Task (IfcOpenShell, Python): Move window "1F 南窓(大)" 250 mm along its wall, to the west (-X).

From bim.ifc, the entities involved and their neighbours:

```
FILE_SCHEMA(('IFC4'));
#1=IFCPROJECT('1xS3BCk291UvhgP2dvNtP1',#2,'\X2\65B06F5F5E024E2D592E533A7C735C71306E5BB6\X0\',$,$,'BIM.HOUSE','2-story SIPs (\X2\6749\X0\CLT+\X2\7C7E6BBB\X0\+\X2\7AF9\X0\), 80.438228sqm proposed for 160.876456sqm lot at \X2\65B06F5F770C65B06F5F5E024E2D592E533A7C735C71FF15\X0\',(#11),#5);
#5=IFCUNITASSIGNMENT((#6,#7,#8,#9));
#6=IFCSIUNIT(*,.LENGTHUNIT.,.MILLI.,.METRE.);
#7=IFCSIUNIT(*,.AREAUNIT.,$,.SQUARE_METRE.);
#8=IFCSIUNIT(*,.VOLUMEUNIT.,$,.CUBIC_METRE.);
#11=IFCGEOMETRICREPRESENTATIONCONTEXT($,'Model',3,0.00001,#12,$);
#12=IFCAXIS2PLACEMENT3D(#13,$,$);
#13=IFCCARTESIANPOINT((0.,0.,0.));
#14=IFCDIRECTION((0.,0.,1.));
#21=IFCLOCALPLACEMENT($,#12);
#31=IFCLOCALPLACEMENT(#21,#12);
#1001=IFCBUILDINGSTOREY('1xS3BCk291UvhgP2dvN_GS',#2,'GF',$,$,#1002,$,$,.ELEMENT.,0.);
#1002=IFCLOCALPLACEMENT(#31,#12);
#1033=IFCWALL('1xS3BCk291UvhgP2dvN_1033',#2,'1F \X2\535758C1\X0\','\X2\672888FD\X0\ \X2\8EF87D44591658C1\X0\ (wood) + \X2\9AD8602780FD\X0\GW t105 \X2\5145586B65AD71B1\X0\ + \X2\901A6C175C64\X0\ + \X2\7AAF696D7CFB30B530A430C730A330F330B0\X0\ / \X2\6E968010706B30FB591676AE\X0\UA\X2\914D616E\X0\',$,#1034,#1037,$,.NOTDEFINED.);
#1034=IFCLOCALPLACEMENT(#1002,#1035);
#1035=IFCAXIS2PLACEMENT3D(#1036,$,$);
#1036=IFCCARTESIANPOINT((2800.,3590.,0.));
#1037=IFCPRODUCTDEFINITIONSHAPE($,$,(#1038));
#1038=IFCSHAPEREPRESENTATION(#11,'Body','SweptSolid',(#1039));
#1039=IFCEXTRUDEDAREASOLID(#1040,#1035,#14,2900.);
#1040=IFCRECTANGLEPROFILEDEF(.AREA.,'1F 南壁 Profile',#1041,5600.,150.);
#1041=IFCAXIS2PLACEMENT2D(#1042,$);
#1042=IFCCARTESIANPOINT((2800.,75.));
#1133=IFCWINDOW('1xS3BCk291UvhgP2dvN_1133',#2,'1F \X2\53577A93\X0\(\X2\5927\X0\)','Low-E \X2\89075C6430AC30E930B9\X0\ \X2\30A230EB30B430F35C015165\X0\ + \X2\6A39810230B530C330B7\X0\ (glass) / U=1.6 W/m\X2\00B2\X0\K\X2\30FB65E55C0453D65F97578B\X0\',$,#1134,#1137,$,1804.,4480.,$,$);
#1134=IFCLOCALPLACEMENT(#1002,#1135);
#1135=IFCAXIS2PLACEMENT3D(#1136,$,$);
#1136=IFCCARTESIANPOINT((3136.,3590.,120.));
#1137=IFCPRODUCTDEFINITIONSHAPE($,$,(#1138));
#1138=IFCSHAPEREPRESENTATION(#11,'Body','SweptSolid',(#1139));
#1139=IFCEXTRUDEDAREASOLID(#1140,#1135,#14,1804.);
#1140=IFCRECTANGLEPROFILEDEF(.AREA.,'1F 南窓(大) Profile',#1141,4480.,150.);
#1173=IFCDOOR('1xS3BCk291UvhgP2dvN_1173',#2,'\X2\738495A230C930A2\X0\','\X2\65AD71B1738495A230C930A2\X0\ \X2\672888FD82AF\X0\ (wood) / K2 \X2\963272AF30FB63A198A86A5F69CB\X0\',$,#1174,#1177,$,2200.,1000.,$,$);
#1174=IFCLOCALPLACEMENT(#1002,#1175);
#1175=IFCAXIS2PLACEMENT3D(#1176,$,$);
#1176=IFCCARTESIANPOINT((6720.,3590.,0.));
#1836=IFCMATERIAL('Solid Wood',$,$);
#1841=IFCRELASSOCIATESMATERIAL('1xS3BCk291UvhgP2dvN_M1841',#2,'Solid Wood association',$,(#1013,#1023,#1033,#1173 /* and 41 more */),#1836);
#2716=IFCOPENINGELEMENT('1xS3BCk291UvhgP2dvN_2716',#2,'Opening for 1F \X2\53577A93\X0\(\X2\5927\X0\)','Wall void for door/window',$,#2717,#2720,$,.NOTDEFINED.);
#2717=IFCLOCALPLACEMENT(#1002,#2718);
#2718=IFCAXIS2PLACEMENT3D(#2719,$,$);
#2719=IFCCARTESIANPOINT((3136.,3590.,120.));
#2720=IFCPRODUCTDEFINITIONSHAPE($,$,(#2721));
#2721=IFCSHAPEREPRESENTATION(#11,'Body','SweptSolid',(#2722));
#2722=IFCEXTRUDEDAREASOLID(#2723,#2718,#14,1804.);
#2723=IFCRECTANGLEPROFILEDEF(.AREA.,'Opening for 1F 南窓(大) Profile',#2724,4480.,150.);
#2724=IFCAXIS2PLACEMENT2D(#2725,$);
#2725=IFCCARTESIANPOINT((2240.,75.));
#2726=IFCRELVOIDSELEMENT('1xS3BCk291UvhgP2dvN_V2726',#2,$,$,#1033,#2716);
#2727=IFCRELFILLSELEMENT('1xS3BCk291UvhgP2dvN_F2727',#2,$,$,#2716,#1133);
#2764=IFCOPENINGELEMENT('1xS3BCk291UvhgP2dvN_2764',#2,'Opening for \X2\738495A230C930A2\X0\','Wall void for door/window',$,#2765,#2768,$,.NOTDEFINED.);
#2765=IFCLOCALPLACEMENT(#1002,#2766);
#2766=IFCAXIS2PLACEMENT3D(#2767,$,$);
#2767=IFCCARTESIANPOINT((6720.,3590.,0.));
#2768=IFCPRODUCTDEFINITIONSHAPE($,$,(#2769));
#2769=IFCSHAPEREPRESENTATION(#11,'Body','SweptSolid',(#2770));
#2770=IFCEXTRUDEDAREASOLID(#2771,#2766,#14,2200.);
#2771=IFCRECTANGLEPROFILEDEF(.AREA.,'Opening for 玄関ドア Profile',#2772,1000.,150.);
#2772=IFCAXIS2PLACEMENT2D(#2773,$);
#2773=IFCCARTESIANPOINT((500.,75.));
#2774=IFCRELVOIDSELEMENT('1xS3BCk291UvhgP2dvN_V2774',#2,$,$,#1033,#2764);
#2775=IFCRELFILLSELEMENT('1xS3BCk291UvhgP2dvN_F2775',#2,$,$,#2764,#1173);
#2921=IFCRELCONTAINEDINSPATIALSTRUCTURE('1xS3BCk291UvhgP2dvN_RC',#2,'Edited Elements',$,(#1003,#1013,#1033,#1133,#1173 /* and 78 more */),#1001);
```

```python
import ifcopenshell
import ifcopenshell.api.geometry
import ifcopenshell.util.placement

model = ifcopenshell.open("bim.ifc")

window = model.by_id(1133)
opening = window.FillsVoids[0].RelatingOpeningElement
wall = opening.VoidsElements[0].RelatingBuildingElement

wall_matrix = ifcopenshell.util.placement.get_local_placement(wall.ObjectPlacement)
shift = wall_matrix[:3, 0] * -250.0
before = ifcopenshell.util.placement.get_local_placement(window.ObjectPlacement)[:3, 3].copy()

# The window is not placed relative to its opening, so move both.
for product in (opening, window):
    matrix = ifcopenshell.util.placement.get_local_placement(product.ObjectPlacement)
    matrix[:3, 3] += shift
    ifcopenshell.api.geometry.edit_object_placement(model, product=product, matrix=matrix, is_si=False)

after = ifcopenshell.util.placement.get_local_placement(window.ObjectPlacement)[:3, 3]
print("window moved by", (after - before).round(3) + 0.0)

model.write("bim_rev.ifc")
```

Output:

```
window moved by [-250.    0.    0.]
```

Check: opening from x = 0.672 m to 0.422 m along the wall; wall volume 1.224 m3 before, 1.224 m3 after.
